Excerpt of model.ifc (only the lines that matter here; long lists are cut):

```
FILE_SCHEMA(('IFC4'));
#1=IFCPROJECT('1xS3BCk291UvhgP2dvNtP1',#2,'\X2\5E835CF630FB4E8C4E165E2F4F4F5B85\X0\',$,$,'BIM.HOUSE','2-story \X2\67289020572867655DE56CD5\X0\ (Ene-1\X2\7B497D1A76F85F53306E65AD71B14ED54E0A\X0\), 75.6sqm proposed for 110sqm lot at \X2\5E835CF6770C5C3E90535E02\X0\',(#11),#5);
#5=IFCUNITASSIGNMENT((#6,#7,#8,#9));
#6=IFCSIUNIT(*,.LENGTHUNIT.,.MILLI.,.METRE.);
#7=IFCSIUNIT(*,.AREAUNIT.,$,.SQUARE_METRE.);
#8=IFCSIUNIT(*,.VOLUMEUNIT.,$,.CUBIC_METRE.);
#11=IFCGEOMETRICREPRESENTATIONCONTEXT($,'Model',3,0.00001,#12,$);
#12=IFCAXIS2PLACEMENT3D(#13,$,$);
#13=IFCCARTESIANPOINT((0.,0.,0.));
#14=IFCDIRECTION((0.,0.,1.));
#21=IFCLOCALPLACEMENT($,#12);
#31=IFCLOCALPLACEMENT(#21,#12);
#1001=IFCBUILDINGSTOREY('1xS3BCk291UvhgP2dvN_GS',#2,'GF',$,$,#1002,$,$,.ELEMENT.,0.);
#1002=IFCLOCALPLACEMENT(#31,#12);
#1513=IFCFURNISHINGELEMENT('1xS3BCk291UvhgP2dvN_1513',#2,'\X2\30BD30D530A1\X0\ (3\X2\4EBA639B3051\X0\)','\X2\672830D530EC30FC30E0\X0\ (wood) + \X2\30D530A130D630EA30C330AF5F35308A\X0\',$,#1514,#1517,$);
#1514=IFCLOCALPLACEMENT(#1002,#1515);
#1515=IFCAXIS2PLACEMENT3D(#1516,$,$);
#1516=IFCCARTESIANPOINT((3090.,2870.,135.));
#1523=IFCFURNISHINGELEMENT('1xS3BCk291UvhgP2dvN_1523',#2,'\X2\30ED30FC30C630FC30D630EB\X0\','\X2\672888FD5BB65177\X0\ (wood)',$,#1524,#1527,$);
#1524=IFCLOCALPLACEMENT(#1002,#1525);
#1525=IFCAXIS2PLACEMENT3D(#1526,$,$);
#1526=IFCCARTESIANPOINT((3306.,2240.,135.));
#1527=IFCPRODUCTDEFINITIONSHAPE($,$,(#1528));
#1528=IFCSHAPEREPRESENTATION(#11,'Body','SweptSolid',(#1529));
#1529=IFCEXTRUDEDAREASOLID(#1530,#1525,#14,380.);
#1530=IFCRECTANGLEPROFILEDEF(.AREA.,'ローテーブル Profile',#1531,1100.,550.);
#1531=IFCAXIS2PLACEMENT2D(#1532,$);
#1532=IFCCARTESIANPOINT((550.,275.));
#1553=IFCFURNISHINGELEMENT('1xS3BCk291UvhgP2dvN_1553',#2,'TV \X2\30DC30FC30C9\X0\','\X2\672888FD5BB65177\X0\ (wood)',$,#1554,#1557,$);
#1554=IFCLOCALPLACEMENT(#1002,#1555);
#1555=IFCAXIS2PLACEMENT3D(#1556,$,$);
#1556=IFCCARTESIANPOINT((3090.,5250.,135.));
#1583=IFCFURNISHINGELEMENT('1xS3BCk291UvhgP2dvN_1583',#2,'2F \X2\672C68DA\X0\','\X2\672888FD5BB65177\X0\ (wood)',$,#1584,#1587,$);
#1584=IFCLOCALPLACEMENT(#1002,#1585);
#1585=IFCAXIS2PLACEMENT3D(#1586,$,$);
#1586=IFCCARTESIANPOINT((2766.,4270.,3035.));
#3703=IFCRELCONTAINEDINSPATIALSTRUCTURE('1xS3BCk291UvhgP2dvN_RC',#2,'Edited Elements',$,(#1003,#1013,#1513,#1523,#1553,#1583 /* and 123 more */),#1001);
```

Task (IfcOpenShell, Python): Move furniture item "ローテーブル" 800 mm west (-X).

```python
import ifcopenshell
import ifcopenshell.api.geometry
import ifcopenshell.util.placement

model = ifcopenshell.open("model.ifc")

item = model.by_id(1523)
matrix = ifcopenshell.util.placement.get_local_placement(item.ObjectPlacement)
matrix[0, 3] -= 800.0
ifcopenshell.api.geometry.edit_object_placement(model, product=item, matrix=matrix, is_si=False)

print(ifcopenshell.util.placement.get_local_placement(item.ObjectPlacement).round(3) + 0.0)

model.write("model_edited.ifc")
```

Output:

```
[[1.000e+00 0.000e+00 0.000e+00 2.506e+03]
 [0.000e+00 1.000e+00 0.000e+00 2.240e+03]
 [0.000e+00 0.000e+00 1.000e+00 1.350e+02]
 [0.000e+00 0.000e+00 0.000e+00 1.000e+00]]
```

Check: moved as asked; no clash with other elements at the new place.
